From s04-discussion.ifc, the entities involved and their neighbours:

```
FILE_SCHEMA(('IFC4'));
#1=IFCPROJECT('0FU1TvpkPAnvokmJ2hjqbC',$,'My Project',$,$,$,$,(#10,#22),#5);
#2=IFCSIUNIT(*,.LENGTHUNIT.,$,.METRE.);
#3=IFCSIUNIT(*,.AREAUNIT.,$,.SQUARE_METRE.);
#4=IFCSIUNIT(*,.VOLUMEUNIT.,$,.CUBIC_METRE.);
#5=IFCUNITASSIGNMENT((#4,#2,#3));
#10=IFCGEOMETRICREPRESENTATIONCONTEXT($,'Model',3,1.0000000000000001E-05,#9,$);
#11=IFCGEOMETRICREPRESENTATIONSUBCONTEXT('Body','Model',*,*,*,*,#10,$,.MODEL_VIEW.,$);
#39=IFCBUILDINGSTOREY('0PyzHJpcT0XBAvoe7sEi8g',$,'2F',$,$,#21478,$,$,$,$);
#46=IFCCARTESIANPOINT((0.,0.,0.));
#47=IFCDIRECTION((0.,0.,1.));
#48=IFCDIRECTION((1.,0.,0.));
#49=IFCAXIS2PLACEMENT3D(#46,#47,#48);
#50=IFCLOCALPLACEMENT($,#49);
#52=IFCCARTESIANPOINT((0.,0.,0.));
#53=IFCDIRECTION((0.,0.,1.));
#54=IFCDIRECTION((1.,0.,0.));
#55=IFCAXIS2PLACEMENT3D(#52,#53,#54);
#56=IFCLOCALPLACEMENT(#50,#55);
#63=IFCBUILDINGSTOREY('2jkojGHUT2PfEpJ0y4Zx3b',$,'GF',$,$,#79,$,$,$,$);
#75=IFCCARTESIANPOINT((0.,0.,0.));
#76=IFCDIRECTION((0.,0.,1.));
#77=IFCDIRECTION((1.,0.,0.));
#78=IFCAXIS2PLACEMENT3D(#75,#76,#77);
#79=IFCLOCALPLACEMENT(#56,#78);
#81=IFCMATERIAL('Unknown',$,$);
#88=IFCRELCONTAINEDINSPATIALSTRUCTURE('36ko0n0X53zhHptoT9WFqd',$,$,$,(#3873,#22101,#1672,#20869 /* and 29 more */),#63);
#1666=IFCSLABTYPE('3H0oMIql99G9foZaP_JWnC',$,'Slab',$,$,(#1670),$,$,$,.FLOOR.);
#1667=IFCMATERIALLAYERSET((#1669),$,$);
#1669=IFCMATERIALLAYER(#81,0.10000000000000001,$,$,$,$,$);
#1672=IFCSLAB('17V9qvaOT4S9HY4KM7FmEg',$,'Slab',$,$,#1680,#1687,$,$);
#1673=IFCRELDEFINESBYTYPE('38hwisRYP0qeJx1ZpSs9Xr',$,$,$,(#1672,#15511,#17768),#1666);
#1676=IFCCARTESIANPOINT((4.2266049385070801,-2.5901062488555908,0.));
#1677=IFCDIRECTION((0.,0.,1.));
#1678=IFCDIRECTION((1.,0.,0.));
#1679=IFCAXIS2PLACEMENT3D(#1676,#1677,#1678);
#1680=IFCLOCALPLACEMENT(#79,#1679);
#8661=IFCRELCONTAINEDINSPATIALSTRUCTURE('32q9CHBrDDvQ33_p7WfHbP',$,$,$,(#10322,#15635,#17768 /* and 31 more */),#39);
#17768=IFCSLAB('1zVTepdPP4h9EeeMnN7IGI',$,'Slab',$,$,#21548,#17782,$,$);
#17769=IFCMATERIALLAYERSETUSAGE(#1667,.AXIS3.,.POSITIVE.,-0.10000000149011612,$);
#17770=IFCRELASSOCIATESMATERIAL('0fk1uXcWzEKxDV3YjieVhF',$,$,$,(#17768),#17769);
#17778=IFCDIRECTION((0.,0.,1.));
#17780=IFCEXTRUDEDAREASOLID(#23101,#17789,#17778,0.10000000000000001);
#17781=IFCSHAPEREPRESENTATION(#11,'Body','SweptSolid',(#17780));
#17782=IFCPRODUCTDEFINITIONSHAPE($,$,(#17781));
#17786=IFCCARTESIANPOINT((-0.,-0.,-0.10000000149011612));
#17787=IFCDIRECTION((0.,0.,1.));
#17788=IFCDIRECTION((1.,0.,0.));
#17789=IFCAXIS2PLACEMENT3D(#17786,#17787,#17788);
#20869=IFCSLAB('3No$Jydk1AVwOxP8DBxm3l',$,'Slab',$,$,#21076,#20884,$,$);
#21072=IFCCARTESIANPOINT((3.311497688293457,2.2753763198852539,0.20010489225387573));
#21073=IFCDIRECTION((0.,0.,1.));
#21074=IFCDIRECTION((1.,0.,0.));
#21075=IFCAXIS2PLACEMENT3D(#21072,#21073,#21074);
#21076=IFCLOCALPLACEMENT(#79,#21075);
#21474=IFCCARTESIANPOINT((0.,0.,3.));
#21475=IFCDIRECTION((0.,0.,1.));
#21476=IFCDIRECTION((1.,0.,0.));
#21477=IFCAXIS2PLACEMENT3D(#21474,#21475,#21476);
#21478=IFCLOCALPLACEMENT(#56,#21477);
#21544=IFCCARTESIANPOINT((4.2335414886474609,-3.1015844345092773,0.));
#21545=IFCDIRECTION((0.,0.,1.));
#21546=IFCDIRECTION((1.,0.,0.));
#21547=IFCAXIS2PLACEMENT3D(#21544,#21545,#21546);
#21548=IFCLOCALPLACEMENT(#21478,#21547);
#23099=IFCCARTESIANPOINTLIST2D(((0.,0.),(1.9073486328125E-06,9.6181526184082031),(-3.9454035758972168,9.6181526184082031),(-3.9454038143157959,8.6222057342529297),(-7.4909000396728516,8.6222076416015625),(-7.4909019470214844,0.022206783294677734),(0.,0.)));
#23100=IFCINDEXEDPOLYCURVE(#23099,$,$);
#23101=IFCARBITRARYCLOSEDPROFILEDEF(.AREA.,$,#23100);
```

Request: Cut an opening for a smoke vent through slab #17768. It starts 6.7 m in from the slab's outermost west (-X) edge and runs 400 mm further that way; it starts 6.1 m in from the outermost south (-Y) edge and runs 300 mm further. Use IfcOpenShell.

```python
import numpy as np
import ifcopenshell
import ifcopenshell.api.feature
import ifcopenshell.api.geometry
import ifcopenshell.api.root
import ifcopenshell.geom
import ifcopenshell.util.placement
import ifcopenshell.util.representation
import ifcopenshell.util.shape
import ifcopenshell.util.unit

model = ifcopenshell.open("s04-discussion.ifc")
unit_scale = ifcopenshell.util.unit.calculate_unit_scale(model)
settings = ifcopenshell.geom.settings()


def volume(element):
    """Net volume in cubic metres, openings subtracted."""
    shape = ifcopenshell.geom.create_shape(settings, element)
    return ifcopenshell.util.shape.get_volume(shape.geometry)


slab = model.by_guid("1zVTepdPP4h9EeeMnN7IGI")
before = volume(slab)

# Extent in the slab's own axes, in metres. The edges named are its -X and -Y sides.
slab_shape = ifcopenshell.geom.create_shape(settings, slab)
vertices = ifcopenshell.util.shape.get_vertices(slab_shape.geometry)
x_min, y_min, bottom = vertices.min(axis=0)
top = vertices[:, 2].max()

opening = ifcopenshell.api.root.create_entity(model, ifc_class="IfcOpeningElement", name="Smoke vent opening", predefined_type="OPENING")
context = ifcopenshell.util.representation.get_context(model, "Model", "Body", "MODEL_VIEW")
width, depth = 0.4, 0.3
outline = [(0.0, 0.0), (width, 0.0), (width, depth), (0.0, depth), (0.0, 0.0)]
# Overshoot both faces by 50 mm so the cut is clean.
shape = ifcopenshell.api.geometry.add_slab_representation(
    model, context=context, depth=top - bottom + 0.1, polyline=outline
)
ifcopenshell.api.geometry.assign_representation(model, product=opening, representation=shape)

matrix = ifcopenshell.util.placement.get_local_placement(slab.ObjectPlacement)
matrix[:, 3] = matrix @ np.append(np.array([x_min + 6.7, y_min + 6.1, bottom - 0.05]) / unit_scale, 1.0)
ifcopenshell.api.geometry.edit_object_placement(model, product=opening, matrix=matrix, is_si=False)
ifcopenshell.api.feature.add_feature(model, feature=opening, element=slab)

after = volume(slab)

print(f"slab volume {before:.3f} -> {after:.3f} m3")

model.write("s04-discussion_edited.ifc")
```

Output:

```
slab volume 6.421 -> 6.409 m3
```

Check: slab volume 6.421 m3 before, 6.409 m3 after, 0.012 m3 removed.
